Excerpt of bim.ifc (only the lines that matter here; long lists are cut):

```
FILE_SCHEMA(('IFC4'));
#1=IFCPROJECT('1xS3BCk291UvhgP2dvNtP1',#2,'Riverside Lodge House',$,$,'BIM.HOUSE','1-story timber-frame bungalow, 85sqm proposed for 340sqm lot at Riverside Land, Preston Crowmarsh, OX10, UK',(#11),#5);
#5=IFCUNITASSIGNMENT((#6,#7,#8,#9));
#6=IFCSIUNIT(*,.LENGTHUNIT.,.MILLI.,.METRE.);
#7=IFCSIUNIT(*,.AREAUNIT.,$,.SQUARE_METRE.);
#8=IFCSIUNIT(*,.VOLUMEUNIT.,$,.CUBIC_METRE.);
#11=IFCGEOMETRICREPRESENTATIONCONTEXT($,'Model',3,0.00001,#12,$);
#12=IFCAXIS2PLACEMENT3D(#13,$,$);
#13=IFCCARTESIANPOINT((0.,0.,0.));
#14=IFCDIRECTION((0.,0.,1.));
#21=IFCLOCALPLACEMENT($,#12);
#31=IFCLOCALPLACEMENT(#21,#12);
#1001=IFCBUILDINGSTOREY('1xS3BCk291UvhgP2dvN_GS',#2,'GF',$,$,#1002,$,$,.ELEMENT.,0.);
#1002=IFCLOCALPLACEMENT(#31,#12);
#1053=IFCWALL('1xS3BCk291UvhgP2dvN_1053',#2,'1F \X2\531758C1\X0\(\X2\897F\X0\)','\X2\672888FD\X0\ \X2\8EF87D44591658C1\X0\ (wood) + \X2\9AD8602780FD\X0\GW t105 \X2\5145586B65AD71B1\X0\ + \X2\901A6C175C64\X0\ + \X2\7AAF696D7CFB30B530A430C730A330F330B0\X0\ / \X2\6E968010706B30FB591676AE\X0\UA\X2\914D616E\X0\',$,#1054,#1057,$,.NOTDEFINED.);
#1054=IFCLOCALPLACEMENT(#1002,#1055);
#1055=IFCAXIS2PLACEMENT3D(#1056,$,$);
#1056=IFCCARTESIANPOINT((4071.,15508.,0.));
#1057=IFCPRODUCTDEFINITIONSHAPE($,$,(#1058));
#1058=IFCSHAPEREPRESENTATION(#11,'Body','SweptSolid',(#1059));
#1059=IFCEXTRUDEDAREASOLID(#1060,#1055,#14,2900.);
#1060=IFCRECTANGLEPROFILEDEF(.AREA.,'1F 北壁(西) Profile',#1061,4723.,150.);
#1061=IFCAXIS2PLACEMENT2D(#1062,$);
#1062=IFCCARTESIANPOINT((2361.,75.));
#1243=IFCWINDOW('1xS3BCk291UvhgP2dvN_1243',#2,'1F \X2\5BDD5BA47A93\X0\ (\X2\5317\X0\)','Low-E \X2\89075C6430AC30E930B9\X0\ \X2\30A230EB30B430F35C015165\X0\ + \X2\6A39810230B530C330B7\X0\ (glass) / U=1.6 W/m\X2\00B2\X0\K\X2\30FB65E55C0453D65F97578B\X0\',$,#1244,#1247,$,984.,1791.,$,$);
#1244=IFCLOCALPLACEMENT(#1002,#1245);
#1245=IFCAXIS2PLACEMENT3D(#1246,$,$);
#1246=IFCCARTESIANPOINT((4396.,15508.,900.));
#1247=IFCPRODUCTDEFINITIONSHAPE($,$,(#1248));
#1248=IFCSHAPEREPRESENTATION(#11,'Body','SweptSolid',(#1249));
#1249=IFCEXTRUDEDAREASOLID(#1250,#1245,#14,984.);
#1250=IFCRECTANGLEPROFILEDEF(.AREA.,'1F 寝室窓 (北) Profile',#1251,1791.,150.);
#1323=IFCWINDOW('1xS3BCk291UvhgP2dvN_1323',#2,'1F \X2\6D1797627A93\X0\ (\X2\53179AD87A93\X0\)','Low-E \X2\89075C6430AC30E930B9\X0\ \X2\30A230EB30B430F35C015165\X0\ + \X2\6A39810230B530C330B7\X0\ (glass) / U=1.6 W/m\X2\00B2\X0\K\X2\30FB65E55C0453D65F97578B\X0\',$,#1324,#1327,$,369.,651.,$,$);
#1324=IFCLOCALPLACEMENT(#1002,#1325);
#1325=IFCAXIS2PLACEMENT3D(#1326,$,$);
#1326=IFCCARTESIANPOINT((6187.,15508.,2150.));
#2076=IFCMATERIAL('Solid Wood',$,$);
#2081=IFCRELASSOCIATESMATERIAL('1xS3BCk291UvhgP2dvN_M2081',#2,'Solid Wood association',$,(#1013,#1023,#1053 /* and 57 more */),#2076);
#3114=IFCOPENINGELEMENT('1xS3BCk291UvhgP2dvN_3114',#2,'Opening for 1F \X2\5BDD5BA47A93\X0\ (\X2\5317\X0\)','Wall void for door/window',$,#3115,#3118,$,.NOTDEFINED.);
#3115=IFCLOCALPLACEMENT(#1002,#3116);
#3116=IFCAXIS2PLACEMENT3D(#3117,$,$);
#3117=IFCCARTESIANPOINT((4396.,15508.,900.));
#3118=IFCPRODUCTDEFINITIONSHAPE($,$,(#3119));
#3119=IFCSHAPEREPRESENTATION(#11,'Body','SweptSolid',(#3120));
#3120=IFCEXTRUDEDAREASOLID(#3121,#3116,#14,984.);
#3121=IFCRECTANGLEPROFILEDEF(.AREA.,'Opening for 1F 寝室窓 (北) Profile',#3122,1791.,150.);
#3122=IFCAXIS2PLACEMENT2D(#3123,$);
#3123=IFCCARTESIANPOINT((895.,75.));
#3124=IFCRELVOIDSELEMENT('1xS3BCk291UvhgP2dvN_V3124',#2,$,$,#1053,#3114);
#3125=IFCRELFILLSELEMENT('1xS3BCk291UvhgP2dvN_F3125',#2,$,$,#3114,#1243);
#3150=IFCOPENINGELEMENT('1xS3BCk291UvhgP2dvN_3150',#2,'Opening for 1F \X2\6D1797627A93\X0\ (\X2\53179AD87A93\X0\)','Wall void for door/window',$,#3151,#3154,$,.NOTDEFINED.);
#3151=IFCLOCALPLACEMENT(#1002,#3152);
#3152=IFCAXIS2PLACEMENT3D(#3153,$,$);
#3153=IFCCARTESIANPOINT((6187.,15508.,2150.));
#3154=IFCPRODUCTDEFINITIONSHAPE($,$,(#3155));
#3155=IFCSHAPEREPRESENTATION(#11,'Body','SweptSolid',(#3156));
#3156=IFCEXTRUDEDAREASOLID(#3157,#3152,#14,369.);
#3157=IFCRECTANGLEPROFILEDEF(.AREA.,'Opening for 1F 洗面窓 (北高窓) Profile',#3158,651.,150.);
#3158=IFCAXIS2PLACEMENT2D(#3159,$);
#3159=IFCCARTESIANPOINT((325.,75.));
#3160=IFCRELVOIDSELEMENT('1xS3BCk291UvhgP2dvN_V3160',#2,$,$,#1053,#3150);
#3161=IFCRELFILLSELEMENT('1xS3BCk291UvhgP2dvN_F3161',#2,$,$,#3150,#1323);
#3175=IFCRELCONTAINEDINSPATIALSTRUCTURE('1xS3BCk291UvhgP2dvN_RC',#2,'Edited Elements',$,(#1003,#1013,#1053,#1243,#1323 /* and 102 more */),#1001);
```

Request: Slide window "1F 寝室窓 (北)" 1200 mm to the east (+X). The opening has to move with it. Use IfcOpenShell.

```python
import ifcopenshell
import ifcopenshell.api.geometry
import ifcopenshell.util.placement

model = ifcopenshell.open("bim.ifc")

window = model.by_id(1243)
opening = window.FillsVoids[0].RelatingOpeningElement
wall = opening.VoidsElements[0].RelatingBuildingElement

wall_matrix = ifcopenshell.util.placement.get_local_placement(wall.ObjectPlacement)
shift = wall_matrix[:3, 0] * 1200.0
before = ifcopenshell.util.placement.get_local_placement(window.ObjectPlacement)[:3, 3].copy()

# The window is not placed relative to its opening, so move both.
for product in (opening, window):
    matrix = ifcopenshell.util.placement.get_local_placement(product.ObjectPlacement)
    matrix[:3, 3] += shift
    ifcopenshell.api.geometry.edit_object_placement(model, product=product, matrix=matrix, is_si=False)

after = ifcopenshell.util.placement.get_local_placement(window.ObjectPlacement)[:3, 3]
print("window moved by", (after - before).round(3) + 0.0)

model.write("bim_updated.ifc")
```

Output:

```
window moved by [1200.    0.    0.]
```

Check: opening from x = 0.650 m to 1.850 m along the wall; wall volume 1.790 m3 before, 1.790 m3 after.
